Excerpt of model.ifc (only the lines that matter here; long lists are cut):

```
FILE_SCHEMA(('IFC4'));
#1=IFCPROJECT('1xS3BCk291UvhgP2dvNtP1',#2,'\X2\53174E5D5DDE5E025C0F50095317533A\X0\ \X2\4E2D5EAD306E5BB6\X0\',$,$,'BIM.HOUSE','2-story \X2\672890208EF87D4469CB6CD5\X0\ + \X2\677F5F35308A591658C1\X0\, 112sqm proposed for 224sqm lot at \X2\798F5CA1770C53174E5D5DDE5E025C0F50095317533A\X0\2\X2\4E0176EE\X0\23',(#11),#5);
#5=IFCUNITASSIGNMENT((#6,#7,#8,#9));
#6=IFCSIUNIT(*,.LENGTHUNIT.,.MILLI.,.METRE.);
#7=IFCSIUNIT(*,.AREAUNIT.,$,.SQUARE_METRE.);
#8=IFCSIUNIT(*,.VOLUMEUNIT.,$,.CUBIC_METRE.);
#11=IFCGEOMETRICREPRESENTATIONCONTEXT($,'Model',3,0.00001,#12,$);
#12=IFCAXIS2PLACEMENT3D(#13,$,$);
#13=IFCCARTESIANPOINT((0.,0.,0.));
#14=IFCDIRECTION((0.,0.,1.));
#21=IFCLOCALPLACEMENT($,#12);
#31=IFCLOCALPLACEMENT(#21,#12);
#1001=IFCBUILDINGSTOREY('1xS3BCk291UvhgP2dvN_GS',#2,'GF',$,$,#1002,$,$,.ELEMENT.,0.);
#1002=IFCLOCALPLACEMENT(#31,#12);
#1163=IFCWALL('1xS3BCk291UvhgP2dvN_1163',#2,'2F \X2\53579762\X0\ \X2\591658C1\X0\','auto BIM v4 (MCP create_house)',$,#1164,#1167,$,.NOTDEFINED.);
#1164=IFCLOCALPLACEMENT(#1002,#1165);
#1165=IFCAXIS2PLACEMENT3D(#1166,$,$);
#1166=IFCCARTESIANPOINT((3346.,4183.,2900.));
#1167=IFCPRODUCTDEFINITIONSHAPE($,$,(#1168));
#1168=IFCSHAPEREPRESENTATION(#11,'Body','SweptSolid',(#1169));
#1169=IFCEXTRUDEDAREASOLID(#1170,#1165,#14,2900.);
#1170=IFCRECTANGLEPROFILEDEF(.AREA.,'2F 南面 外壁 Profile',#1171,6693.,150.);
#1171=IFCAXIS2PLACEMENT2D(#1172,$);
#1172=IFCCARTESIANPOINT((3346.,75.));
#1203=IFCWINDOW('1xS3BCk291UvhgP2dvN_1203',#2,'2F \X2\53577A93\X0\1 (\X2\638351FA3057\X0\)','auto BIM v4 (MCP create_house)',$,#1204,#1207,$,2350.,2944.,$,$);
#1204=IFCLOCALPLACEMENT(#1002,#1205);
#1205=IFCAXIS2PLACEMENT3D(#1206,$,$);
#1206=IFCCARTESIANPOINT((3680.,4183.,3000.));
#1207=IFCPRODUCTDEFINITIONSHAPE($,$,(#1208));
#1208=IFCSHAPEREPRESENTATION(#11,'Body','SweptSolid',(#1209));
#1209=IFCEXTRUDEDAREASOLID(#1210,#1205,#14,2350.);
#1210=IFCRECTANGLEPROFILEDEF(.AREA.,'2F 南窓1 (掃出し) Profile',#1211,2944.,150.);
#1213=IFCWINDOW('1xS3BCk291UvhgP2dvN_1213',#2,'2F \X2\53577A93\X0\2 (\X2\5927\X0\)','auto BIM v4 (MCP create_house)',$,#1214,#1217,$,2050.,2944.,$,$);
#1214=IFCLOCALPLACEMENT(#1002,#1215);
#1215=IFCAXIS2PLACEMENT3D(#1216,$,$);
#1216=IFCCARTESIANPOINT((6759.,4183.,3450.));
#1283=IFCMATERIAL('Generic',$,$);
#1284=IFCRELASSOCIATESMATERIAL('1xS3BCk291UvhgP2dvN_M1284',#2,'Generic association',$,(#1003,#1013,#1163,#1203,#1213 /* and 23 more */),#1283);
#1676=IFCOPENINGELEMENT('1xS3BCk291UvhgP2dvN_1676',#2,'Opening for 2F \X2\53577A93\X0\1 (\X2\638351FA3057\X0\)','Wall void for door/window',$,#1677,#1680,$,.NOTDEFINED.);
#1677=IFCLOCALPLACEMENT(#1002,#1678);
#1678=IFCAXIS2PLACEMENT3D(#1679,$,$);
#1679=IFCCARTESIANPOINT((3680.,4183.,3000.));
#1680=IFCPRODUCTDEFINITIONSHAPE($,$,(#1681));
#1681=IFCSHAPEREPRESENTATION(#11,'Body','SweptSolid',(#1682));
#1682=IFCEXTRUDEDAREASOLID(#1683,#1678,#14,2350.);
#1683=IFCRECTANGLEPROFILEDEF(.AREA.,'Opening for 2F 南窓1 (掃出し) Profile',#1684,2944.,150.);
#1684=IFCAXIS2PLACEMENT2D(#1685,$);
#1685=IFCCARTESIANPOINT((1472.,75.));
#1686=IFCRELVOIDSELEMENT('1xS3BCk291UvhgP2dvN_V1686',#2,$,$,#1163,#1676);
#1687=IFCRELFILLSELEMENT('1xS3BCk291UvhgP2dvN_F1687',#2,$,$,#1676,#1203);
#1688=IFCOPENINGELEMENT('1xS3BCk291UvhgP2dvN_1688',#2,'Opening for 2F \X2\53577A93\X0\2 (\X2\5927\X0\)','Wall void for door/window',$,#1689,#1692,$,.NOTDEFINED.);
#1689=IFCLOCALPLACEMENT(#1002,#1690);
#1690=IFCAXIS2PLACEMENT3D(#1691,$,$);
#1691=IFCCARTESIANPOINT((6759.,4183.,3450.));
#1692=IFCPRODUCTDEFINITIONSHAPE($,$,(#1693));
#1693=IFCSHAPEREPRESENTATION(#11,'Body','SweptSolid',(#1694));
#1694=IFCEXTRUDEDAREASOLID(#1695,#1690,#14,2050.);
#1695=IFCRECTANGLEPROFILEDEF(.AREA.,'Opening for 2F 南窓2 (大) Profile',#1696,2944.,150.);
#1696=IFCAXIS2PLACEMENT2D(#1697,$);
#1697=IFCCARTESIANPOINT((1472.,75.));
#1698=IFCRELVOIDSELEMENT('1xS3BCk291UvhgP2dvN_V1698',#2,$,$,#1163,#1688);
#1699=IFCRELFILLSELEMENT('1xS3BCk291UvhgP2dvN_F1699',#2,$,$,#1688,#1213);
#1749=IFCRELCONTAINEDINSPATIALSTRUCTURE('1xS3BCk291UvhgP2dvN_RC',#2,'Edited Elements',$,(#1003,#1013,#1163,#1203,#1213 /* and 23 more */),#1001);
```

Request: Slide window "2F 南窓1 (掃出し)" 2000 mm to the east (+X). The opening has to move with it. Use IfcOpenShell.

```python
import ifcopenshell
import ifcopenshell.api.geometry
import ifcopenshell.util.placement
import ifcopenshell.util.unit

model = ifcopenshell.open("model.ifc")
unit_scale = ifcopenshell.util.unit.calculate_unit_scale(model)

window = model.by_guid("1xS3BCk291UvhgP2dvN_1203")
opening = window.FillsVoids[0].RelatingOpeningElement
wall = opening.VoidsElements[0].RelatingBuildingElement

wall_matrix = ifcopenshell.util.placement.get_local_placement(wall.ObjectPlacement)
shift = wall_matrix[:3, 0] * 2 / unit_scale
before = ifcopenshell.util.placement.get_local_placement(window.ObjectPlacement)[:3, 3].copy()

# The window is not placed relative to its opening, so move both.
for product in (opening, window):
    matrix = ifcopenshell.util.placement.get_local_placement(product.ObjectPlacement)
    matrix[:3, 3] += shift
    ifcopenshell.api.geometry.edit_object_placement(model, product=product, matrix=matrix, is_si=False)

after = ifcopenshell.util.placement.get_local_placement(window.ObjectPlacement)[:3, 3]
print("window moved by", (after - before).round(3) + 0.0)

model.write("model-out.ifc")
```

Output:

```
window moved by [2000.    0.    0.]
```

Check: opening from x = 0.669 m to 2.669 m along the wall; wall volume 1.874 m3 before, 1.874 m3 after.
